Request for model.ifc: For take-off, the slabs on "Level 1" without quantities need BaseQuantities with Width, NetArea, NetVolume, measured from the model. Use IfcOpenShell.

First a look at what the model holds.

```python
import ifcopenshell
import ifcopenshell.util.element
import ifcopenshell.util.unit

model = ifcopenshell.open("model.ifc")
print(model.schema)
for unit_type in ("LENGTHUNIT", "AREAUNIT", "VOLUMEUNIT"):
    print(unit_type, ifcopenshell.util.unit.calculate_unit_scale(model, unit_type))
storey = next(s for s in model.by_type("IfcBuildingStorey") if s.Name == "Level 1")
slabs = [e for e in ifcopenshell.util.element.get_decomposition(storey) if e.is_a("IfcSlab")]
for e in sorted(slabs, key=lambda e: e.id()):
    print(e.id(), e.is_a(), e.Name, list(ifcopenshell.util.element.get_psets(e, qtos_only=True)), sep=" | ")
```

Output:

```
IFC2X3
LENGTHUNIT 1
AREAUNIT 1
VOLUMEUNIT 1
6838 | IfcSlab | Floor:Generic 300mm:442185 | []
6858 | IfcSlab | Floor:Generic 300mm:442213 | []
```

```python
import ifcopenshell
import ifcopenshell.api.pset
import ifcopenshell.geom
import ifcopenshell.util.element
import ifcopenshell.util.shape
import ifcopenshell.util.unit

model = ifcopenshell.open("model.ifc")
unit_scale = ifcopenshell.util.unit.calculate_unit_scale(model)
area_scale = ifcopenshell.util.unit.calculate_unit_scale(model, "AREAUNIT")
volume_scale = ifcopenshell.util.unit.calculate_unit_scale(model, "VOLUMEUNIT")
settings = ifcopenshell.geom.settings()

storey = next(s for s in model.by_type("IfcBuildingStorey") if s.Name == "Level 1")
slabs = [e for e in ifcopenshell.util.element.get_decomposition(storey) if e.is_a("IfcSlab")]

for e in sorted(slabs, key=lambda e: e.id()):
    if ifcopenshell.util.element.get_psets(e, qtos_only=True, should_inherit=False):
        continue
    # Geometry comes back in metres, in the element's own axes.
    shape = ifcopenshell.geom.create_shape(settings, e)
    values = {
        "Width": ifcopenshell.util.shape.get_z(shape.geometry) / unit_scale,
        "NetArea": ifcopenshell.util.shape.get_footprint_area(shape.geometry) / area_scale,
        "NetVolume": ifcopenshell.util.shape.get_volume(shape.geometry) / volume_scale,
    }
    qto = ifcopenshell.api.pset.add_qto(model, product=e, name="BaseQuantities")
    ifcopenshell.api.pset.edit_qto(model, qto=qto, properties=values)
    print(e.id(), {k: round(v, 3) for k, v in values.items()})

model.write("model_rev.ifc")
```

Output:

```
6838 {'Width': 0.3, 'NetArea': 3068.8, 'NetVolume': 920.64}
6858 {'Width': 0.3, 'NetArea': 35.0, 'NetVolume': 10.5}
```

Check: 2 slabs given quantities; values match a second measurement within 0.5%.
